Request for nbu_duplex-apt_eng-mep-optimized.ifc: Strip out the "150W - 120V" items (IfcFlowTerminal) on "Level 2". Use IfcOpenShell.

First a look at what the model holds.

```python
import ifcopenshell
import ifcopenshell.util.element

model = ifcopenshell.open("nbu_duplex-apt_eng-mep-optimized.ifc")
print(model.schema)
storey = next(s for s in model.by_type("IfcBuildingStorey") if s.Name == "Level 2")
terminals = [e for e in ifcopenshell.util.element.get_decomposition(storey) if e.is_a("IfcFlowTerminal")]
seen = {}
for e in terminals:
    element_type = ifcopenshell.util.element.get_type(e)
    name = element_type.Name if element_type not in (None, e) else None
    seen[name] = seen.get(name, 0) + 1
for name, count in sorted(seen.items(), key=str):
    print(count, "x", name)
```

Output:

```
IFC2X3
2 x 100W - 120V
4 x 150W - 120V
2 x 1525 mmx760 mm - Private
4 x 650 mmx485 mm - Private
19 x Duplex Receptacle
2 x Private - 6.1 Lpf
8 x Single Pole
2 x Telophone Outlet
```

```python
import ifcopenshell
import ifcopenshell.api.root
import ifcopenshell.util.element

model = ifcopenshell.open("nbu_duplex-apt_eng-mep-optimized.ifc")

storey = next(s for s in model.by_type("IfcBuildingStorey") if s.Name == "Level 2")
terminals = [e for e in ifcopenshell.util.element.get_decomposition(storey) if e.is_a("IfcFlowTerminal")]
targets = [e for e in terminals if (t := ifcopenshell.util.element.get_type(e)) not in (None, e) and t.Name == "150W - 120V"]

for e in targets:
    ifcopenshell.api.root.remove_product(model, product=e)
print(len(targets), "removed")

model.write("nbu_duplex-apt_eng-mep-optimized_updated.ifc")
```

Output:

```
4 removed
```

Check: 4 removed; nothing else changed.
